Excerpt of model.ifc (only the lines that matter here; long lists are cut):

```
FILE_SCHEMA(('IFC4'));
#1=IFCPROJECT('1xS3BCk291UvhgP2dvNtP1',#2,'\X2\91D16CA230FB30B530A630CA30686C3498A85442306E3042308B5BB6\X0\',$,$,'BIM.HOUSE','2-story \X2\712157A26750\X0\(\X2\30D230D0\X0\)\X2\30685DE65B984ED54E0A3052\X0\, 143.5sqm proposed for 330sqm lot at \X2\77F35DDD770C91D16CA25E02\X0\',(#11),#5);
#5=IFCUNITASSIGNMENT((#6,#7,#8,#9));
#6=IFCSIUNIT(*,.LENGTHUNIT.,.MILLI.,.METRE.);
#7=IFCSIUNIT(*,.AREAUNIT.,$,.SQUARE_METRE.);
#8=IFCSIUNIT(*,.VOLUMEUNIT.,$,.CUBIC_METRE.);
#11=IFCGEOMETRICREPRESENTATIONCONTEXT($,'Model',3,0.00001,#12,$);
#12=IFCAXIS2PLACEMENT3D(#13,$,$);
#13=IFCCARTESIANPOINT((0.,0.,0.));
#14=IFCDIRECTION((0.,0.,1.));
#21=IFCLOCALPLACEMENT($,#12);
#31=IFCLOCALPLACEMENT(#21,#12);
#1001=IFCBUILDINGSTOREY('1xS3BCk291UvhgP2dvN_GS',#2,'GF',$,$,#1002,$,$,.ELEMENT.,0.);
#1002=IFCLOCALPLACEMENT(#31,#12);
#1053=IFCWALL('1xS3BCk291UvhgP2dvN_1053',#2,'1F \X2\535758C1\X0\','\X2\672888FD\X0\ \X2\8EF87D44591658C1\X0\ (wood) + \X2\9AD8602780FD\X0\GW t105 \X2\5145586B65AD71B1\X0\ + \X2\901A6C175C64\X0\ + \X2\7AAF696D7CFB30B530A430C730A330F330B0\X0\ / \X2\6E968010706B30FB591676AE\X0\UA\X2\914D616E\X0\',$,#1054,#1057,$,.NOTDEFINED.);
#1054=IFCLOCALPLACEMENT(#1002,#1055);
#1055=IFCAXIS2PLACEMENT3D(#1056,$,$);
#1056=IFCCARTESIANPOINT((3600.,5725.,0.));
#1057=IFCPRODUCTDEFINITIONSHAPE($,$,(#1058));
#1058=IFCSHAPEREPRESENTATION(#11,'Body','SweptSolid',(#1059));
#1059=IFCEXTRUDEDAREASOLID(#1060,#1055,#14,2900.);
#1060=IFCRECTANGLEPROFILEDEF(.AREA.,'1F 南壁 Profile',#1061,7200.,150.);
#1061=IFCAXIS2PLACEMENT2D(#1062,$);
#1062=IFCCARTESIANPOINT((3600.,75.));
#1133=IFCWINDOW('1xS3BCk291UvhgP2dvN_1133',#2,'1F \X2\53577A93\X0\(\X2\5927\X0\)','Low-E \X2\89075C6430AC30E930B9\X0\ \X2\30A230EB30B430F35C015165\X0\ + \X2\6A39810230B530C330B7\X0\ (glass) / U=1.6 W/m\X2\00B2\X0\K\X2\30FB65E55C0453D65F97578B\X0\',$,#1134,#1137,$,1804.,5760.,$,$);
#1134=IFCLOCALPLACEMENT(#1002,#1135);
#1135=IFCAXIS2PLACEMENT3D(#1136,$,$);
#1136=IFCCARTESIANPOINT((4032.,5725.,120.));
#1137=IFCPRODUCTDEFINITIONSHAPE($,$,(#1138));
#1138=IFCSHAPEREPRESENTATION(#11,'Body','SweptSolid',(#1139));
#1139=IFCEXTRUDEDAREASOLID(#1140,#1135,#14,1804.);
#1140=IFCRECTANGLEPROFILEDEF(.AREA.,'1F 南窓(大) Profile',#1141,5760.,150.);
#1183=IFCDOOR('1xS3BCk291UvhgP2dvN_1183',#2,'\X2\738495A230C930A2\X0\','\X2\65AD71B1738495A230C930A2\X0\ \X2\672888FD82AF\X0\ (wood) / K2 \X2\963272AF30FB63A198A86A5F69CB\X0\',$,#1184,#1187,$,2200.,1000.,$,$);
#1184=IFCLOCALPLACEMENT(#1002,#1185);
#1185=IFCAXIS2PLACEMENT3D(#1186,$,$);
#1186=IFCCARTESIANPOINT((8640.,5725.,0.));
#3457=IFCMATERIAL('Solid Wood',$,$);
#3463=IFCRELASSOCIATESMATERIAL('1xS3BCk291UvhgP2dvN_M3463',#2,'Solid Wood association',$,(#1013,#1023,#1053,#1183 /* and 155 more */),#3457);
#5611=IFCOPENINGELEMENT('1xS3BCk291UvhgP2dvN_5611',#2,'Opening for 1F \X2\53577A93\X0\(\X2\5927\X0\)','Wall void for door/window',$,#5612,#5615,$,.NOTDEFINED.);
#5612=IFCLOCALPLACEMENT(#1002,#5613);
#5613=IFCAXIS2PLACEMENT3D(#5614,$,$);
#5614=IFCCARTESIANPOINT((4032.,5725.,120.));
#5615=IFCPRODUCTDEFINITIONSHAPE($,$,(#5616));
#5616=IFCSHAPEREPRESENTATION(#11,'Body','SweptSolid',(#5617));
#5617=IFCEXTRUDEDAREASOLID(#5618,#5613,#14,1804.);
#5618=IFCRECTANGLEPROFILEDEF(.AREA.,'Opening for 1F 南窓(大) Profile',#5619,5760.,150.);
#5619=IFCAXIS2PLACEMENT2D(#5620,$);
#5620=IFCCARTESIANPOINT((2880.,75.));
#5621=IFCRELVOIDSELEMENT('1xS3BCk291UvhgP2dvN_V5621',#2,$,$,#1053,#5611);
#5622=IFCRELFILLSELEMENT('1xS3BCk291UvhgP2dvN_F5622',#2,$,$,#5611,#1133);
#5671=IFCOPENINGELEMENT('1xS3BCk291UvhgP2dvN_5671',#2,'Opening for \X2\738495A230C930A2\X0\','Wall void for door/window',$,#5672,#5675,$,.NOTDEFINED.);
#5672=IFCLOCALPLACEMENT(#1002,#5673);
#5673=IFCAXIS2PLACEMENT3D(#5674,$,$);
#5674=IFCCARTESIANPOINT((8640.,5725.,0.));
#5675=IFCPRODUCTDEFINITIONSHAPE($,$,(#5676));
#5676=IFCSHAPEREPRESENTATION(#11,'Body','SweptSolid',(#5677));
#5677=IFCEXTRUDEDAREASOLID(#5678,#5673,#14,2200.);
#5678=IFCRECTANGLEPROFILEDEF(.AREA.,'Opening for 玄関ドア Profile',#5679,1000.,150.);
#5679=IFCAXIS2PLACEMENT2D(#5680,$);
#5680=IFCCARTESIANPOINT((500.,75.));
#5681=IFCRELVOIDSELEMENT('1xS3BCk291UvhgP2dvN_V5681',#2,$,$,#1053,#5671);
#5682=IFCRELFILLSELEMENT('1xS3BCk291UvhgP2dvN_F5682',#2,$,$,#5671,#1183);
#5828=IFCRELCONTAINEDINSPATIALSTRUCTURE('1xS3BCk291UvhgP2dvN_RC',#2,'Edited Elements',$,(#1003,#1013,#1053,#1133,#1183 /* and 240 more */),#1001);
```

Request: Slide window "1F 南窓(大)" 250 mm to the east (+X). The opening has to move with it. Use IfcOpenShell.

```python
import ifcopenshell
import ifcopenshell.api.geometry
import ifcopenshell.util.placement
import ifcopenshell.util.unit

model = ifcopenshell.open("model.ifc")
unit_scale = ifcopenshell.util.unit.calculate_unit_scale(model)

window = model.by_guid("1xS3BCk291UvhgP2dvN_1133")
opening = window.FillsVoids[0].RelatingOpeningElement
wall = opening.VoidsElements[0].RelatingBuildingElement

wall_matrix = ifcopenshell.util.placement.get_local_placement(wall.ObjectPlacement)
shift = wall_matrix[:3, 0] * 0.25 / unit_scale
before = ifcopenshell.util.placement.get_local_placement(window.ObjectPlacement)[:3, 3].copy()

# The window is not placed relative to its opening, so move both.
for product in (opening, window):
    matrix = ifcopenshell.util.placement.get_local_placement(product.ObjectPlacement)
    matrix[:3, 3] += shift
    ifcopenshell.api.geometry.edit_object_placement(model, product=product, matrix=matrix, is_si=False)

after = ifcopenshell.util.placement.get_local_placement(window.ObjectPlacement)[:3, 3]
print("window moved by", (after - before).round(3) + 0.0)

model.write("model_updated.ifc")
```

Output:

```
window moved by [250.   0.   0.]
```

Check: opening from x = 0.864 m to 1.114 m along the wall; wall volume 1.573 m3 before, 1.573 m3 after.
